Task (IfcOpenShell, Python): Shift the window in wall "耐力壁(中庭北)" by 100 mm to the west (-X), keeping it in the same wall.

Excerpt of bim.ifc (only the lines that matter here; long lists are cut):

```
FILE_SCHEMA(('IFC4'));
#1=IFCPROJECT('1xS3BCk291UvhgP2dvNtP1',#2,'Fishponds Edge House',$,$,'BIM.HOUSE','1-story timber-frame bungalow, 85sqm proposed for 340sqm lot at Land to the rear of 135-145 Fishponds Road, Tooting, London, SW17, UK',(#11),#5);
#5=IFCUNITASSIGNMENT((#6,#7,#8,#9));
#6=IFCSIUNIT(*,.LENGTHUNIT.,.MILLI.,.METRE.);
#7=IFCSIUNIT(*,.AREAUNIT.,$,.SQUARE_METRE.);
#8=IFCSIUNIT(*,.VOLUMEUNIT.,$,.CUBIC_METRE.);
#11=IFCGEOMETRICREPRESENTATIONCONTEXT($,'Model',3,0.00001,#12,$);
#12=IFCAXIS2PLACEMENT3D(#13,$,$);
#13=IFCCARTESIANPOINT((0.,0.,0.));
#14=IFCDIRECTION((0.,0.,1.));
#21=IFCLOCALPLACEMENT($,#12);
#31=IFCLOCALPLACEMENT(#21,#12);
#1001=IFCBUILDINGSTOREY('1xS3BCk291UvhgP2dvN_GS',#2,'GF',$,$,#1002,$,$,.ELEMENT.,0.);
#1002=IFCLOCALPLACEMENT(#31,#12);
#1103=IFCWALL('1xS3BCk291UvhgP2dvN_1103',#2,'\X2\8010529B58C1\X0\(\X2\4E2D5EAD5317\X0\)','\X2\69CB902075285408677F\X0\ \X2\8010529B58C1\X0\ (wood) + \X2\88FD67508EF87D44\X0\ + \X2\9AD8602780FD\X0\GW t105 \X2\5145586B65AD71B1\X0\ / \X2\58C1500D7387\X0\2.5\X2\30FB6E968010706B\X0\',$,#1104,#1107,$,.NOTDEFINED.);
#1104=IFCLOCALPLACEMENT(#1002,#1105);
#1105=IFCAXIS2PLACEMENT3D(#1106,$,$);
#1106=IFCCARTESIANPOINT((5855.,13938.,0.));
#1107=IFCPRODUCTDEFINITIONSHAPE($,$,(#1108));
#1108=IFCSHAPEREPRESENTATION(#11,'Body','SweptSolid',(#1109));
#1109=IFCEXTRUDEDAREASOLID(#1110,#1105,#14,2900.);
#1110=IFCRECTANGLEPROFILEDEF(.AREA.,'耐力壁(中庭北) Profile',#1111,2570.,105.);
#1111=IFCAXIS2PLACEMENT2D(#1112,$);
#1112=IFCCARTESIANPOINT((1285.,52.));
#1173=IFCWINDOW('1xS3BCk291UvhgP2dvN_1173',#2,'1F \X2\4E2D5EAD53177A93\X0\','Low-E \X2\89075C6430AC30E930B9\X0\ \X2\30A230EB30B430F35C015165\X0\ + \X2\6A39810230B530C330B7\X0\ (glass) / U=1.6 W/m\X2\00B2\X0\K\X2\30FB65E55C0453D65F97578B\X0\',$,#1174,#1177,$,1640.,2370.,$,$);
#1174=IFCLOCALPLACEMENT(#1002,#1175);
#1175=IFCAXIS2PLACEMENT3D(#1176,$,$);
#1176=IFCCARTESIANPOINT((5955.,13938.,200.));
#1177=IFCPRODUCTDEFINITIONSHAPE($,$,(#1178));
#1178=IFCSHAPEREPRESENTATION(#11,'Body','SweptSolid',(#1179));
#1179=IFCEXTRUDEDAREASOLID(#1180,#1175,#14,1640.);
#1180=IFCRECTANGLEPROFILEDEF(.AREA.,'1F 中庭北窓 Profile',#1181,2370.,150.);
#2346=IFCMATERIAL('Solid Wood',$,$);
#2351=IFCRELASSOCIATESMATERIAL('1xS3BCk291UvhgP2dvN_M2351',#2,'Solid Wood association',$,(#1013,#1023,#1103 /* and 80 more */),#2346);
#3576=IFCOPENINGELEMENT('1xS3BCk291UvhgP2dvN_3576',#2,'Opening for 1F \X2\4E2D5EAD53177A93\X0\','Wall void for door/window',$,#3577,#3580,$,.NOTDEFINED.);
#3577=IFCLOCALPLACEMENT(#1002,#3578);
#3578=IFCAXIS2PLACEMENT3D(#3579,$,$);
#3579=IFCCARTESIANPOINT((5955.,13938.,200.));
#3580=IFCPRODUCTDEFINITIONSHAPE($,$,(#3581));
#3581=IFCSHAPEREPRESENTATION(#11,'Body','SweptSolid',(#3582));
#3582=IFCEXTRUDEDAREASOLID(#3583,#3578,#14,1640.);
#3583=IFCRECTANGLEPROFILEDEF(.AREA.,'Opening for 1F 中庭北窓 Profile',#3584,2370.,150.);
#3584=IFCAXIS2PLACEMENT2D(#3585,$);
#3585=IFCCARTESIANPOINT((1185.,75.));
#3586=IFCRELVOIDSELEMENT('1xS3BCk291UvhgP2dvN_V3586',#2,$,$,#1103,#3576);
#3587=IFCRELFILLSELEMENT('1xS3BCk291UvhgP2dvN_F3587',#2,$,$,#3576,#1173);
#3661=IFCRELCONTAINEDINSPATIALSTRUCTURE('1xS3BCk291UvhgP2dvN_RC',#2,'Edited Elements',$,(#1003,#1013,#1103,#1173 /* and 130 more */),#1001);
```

```python
import ifcopenshell
import ifcopenshell.api.geometry
import ifcopenshell.util.placement

model = ifcopenshell.open("bim.ifc")

window = model.by_guid("1xS3BCk291UvhgP2dvN_1173")
opening = window.FillsVoids[0].RelatingOpeningElement
wall = opening.VoidsElements[0].RelatingBuildingElement

wall_matrix = ifcopenshell.util.placement.get_local_placement(wall.ObjectPlacement)
shift = wall_matrix[:3, 0] * -100.0
before = ifcopenshell.util.placement.get_local_placement(window.ObjectPlacement)[:3, 3].copy()

# The window is not placed relative to its opening, so move both.
for product in (opening, window):
    matrix = ifcopenshell.util.placement.get_local_placement(product.ObjectPlacement)
    matrix[:3, 3] += shift
    ifcopenshell.api.geometry.edit_object_placement(model, product=product, matrix=matrix, is_si=False)

after = ifcopenshell.util.placement.get_local_placement(window.ObjectPlacement)[:3, 3]
print("window moved by", (after - before).round(3) + 0.0)

model.write("bim_updated.ifc")
```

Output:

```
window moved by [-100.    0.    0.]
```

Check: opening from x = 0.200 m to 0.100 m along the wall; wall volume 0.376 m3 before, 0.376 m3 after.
